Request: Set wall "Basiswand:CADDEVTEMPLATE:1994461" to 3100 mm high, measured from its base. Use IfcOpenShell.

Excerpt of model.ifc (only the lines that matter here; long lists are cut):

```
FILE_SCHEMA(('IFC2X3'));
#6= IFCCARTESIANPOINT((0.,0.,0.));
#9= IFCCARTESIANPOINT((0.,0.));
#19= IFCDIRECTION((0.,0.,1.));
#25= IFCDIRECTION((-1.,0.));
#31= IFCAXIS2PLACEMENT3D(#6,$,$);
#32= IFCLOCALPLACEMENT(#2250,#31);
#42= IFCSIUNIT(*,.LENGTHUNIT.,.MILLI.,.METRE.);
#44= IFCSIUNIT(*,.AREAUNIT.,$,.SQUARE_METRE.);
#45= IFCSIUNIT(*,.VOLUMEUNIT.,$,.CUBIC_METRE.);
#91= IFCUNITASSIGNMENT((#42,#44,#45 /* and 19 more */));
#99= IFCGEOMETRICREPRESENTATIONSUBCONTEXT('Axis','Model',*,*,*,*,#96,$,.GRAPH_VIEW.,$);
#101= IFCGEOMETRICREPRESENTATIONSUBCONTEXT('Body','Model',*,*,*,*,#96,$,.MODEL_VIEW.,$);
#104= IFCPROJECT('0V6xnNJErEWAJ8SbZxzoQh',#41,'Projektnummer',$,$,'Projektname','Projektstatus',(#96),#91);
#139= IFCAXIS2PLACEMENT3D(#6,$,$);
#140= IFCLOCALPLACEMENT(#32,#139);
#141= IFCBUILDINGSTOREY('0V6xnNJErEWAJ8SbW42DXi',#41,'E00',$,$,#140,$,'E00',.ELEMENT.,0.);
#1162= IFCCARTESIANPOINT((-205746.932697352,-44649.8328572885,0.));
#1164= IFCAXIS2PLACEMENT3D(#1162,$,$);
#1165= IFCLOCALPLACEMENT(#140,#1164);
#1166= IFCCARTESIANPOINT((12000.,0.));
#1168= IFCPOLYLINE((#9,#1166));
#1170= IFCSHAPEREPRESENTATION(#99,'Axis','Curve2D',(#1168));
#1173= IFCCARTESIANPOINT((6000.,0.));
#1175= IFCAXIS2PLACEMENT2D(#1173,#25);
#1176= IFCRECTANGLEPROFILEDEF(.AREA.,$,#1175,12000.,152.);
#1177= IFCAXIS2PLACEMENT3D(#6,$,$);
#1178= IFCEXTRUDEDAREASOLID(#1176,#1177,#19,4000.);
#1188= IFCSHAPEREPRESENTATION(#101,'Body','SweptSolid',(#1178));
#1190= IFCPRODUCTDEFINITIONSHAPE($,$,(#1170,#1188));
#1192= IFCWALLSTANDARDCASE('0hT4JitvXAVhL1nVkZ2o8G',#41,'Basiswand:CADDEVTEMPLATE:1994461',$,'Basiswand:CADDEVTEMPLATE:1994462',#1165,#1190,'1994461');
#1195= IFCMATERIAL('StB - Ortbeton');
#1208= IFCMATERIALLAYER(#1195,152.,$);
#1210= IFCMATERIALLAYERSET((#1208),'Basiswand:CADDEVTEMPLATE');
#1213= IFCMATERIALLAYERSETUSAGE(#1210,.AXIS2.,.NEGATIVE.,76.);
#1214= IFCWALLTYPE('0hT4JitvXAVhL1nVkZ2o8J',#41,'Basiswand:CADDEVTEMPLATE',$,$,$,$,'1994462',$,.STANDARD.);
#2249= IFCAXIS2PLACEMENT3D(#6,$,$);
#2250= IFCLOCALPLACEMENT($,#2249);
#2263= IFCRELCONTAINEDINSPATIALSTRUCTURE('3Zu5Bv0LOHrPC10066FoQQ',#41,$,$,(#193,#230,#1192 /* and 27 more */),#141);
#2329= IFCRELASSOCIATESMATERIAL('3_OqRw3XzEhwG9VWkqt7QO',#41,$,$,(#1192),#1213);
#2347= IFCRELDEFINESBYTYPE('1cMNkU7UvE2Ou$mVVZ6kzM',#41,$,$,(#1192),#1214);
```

```python
import ifcopenshell
import ifcopenshell.geom
import ifcopenshell.util.representation
import ifcopenshell.util.shape
import ifcopenshell.util.unit

model = ifcopenshell.open("model.ifc")
unit_scale = ifcopenshell.util.unit.calculate_unit_scale(model)
settings = ifcopenshell.geom.settings()


def volume(element):
    """Net volume in cubic metres, openings subtracted."""
    shape = ifcopenshell.geom.create_shape(settings, element)
    return ifcopenshell.util.shape.get_volume(shape.geometry)


wall = model.by_guid("0hT4JitvXAVhL1nVkZ2o8G")
before = volume(wall)

body = ifcopenshell.util.representation.get_representation(wall, "Model", "Body")
solid = body.Items[0]
old_height = solid.Depth
solid.Depth = 3.1 / unit_scale
after = volume(wall)

print(f"height {old_height:g} -> {solid.Depth:g}, volume {before:.3f} -> {after:.3f} m3")

model.write("model_rev.ifc")
```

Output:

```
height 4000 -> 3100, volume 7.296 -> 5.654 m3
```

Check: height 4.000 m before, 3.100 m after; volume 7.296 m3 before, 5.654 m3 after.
